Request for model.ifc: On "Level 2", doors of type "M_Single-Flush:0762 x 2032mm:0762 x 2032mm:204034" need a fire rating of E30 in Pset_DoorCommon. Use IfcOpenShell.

First a look at what the model holds.

```python
import ifcopenshell
import ifcopenshell.util.element

model = ifcopenshell.open("model.ifc")
print(model.schema)
storey = next(s for s in model.by_type("IfcBuildingStorey") if s.Name == "Level 2")
doors = [e for e in ifcopenshell.util.element.get_decomposition(storey) if e.is_a("IfcDoor")]
seen = {}
for e in doors:
    element_type = ifcopenshell.util.element.get_type(e)
    key = (element_type.Name if element_type != e and element_type else None, ifcopenshell.util.element.get_pset(e, "Pset_DoorCommon", "FireRating"))
    seen[key] = seen.get(key, 0) + 1
for (name, value), count in sorted(seen.items(), key=str):
    print(count, "x", name, "|", value)
```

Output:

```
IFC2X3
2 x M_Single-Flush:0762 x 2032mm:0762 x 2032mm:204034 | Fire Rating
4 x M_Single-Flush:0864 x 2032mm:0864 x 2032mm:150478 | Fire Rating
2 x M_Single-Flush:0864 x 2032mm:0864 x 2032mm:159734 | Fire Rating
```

```python
import ifcopenshell
import ifcopenshell.api.pset
import ifcopenshell.util.element

model = ifcopenshell.open("model.ifc")

storey = next(s for s in model.by_type("IfcBuildingStorey") if s.Name == "Level 2")
doors = [e for e in ifcopenshell.util.element.get_decomposition(storey) if e.is_a("IfcDoor")]

count = 0
for e in doors:
    element_type = ifcopenshell.util.element.get_type(e)
    if element_type in (None, e) or element_type.Name != "M_Single-Flush:0762 x 2032mm:0762 x 2032mm:204034":
        continue
    # add_pset returns the element's existing set when there is one.
    pset = ifcopenshell.api.pset.add_pset(model, product=e, name="Pset_DoorCommon")
    ifcopenshell.api.pset.edit_pset(model, pset=pset, properties={"FireRating": "E30"})
    count += 1

print(count, "doors updated")

model.write("model_rev.ifc")
```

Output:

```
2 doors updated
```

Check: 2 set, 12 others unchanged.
